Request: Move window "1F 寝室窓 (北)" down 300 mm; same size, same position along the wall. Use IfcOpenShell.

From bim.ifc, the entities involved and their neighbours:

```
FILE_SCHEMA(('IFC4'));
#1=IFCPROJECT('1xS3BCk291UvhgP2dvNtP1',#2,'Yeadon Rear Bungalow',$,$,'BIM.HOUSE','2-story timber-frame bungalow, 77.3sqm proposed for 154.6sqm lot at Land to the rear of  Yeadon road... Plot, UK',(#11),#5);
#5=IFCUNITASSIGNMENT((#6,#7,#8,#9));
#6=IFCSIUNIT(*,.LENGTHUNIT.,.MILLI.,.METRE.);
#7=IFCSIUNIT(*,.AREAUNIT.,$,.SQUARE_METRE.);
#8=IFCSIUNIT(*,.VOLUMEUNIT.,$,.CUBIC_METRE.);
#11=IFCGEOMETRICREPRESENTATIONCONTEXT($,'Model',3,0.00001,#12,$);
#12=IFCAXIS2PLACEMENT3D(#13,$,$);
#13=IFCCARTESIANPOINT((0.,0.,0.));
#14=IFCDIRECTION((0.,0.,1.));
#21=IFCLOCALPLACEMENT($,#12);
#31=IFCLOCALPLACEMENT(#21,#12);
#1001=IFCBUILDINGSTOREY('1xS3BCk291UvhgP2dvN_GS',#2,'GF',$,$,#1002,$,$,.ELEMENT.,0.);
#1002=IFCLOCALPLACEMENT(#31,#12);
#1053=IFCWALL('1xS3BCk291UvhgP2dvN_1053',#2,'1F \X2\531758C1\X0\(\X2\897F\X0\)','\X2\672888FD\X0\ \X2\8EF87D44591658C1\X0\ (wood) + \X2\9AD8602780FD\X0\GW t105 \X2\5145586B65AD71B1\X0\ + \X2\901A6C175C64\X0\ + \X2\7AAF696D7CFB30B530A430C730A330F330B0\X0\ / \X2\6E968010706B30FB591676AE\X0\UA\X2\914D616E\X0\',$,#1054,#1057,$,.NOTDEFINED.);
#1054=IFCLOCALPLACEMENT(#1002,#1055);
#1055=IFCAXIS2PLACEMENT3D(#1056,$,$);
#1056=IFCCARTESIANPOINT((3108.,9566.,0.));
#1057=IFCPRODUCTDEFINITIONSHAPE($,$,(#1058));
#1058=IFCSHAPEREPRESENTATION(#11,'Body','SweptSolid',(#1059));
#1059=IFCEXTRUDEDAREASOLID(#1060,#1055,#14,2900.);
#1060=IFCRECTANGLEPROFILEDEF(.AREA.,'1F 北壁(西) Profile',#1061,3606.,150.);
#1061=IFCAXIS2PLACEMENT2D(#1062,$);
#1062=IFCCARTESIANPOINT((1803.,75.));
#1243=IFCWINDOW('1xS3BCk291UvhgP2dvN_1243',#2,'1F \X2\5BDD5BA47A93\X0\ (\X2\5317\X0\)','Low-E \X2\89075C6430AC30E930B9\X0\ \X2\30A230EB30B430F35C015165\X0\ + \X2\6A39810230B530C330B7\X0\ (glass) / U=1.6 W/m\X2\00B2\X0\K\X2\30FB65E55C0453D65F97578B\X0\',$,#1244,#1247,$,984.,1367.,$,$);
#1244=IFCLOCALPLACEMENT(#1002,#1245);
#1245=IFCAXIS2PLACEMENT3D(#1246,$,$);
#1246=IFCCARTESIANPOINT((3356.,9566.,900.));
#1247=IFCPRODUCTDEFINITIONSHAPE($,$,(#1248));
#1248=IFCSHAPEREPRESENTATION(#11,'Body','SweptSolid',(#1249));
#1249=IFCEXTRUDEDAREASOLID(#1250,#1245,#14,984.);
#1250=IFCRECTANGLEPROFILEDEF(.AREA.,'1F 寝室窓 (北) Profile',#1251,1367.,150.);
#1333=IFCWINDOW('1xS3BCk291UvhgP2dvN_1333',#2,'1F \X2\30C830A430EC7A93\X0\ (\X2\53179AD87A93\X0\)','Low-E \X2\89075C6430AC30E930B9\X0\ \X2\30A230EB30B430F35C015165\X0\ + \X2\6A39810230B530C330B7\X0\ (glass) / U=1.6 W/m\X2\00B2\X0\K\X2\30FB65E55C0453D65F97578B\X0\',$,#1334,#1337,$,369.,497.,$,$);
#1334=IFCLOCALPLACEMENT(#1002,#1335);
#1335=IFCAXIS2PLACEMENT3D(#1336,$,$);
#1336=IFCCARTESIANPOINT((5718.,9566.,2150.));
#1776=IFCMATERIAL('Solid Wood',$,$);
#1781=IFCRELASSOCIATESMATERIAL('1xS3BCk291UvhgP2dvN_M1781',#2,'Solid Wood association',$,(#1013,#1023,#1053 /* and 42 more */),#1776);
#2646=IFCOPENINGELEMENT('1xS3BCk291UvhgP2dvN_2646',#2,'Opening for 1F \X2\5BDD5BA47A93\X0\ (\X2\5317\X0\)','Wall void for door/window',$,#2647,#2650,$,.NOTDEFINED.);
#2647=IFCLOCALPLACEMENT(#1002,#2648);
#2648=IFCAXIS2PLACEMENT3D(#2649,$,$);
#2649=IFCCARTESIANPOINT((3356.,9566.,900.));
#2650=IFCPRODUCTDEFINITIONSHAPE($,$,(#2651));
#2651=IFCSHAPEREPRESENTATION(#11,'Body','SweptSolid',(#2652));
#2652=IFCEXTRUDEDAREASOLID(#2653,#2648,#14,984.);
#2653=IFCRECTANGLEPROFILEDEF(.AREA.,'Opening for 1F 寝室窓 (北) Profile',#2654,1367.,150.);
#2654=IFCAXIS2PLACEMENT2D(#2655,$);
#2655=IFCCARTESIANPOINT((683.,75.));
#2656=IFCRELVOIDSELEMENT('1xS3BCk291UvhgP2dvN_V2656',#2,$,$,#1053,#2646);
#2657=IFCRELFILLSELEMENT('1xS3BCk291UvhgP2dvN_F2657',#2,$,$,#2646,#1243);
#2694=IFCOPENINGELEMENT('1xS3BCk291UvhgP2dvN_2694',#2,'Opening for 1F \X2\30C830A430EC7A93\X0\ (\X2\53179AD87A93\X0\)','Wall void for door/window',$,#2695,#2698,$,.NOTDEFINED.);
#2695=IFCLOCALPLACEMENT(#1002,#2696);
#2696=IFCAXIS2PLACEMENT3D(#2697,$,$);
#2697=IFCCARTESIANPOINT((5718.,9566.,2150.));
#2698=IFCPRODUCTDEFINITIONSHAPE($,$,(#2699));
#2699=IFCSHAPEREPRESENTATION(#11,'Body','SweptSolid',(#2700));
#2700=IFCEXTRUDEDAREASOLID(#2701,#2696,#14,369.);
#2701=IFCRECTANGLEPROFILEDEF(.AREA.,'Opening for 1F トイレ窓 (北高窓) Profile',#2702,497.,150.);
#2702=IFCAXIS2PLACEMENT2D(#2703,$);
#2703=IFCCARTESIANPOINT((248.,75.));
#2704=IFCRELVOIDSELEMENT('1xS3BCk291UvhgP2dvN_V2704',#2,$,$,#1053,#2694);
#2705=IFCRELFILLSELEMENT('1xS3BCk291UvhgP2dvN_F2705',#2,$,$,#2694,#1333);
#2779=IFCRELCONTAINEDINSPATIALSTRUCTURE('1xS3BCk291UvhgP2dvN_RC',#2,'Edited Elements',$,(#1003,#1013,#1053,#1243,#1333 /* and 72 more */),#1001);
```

```python
import numpy as np
import ifcopenshell
import ifcopenshell.api.geometry
import ifcopenshell.util.placement
import ifcopenshell.util.unit

model = ifcopenshell.open("bim.ifc")
unit_scale = ifcopenshell.util.unit.calculate_unit_scale(model)

window = model.by_guid("1xS3BCk291UvhgP2dvN_1243")
opening = window.FillsVoids[0].RelatingOpeningElement
dz = -0.3 / unit_scale

shift = np.array([0.0, 0.0, dz])
# The window is not placed relative to its opening, so move both.
for product in (opening, window):
    matrix = ifcopenshell.util.placement.get_local_placement(product.ObjectPlacement)
    matrix[:3, 3] += shift
    ifcopenshell.api.geometry.edit_object_placement(model, product=product, matrix=matrix, is_si=False)

print(f"moved by {dz * unit_scale:+.3f} m")

model.write("bim_edited.ifc")
```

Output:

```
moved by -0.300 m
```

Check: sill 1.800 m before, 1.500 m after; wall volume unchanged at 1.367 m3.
